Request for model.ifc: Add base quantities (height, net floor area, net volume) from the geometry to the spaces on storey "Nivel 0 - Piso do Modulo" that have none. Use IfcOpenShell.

First a look at what the model holds.

```python
import ifcopenshell
import ifcopenshell.util.element
import ifcopenshell.util.unit

model = ifcopenshell.open("model.ifc")
print(model.schema)
for unit_type in ("LENGTHUNIT", "AREAUNIT", "VOLUMEUNIT"):
    print(unit_type, ifcopenshell.util.unit.calculate_unit_scale(model, unit_type))
storey = next(s for s in model.by_type("IfcBuildingStorey") if s.Name == "Nivel 0 - Piso do Modulo")
spaces = [e for e in ifcopenshell.util.element.get_decomposition(storey) if e.is_a("IfcSpace")]
for e in sorted(spaces, key=lambda e: e.id()):
    print(e.id(), e.is_a(), e.Name, list(ifcopenshell.util.element.get_psets(e, qtos_only=True)), sep=" | ")
```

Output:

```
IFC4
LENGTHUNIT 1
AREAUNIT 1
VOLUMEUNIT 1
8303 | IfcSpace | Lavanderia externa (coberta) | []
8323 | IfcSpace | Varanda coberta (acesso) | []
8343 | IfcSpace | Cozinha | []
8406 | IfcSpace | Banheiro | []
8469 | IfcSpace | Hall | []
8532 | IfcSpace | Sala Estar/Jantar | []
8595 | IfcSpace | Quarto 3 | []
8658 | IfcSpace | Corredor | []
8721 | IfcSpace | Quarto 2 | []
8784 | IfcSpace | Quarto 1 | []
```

```python
import ifcopenshell
import ifcopenshell.api.pset
import ifcopenshell.geom
import ifcopenshell.util.element
import ifcopenshell.util.shape
import ifcopenshell.util.unit

model = ifcopenshell.open("model.ifc")
unit_scale = ifcopenshell.util.unit.calculate_unit_scale(model)
area_scale = ifcopenshell.util.unit.calculate_unit_scale(model, "AREAUNIT")
volume_scale = ifcopenshell.util.unit.calculate_unit_scale(model, "VOLUMEUNIT")
settings = ifcopenshell.geom.settings()

storey = next(s for s in model.by_type("IfcBuildingStorey") if s.Name == "Nivel 0 - Piso do Modulo")
spaces = [e for e in ifcopenshell.util.element.get_decomposition(storey) if e.is_a("IfcSpace")]

for e in sorted(spaces, key=lambda e: e.id()):
    if ifcopenshell.util.element.get_psets(e, qtos_only=True, should_inherit=False):
        continue
    # Geometry comes back in metres, in the element's own axes.
    shape = ifcopenshell.geom.create_shape(settings, e)
    values = {
        "Height": ifcopenshell.util.shape.get_z(shape.geometry) / unit_scale,
        "NetFloorArea": ifcopenshell.util.shape.get_footprint_area(shape.geometry) / area_scale,
        "NetVolume": ifcopenshell.util.shape.get_volume(shape.geometry) / volume_scale,
    }
    qto = ifcopenshell.api.pset.add_qto(model, product=e, name="Qto_SpaceBaseQuantities")
    ifcopenshell.api.pset.edit_qto(model, qto=qto, properties=values)
    print(e.id(), {k: round(v, 3) for k, v in values.items()})

model.write("model-out.ifc")
```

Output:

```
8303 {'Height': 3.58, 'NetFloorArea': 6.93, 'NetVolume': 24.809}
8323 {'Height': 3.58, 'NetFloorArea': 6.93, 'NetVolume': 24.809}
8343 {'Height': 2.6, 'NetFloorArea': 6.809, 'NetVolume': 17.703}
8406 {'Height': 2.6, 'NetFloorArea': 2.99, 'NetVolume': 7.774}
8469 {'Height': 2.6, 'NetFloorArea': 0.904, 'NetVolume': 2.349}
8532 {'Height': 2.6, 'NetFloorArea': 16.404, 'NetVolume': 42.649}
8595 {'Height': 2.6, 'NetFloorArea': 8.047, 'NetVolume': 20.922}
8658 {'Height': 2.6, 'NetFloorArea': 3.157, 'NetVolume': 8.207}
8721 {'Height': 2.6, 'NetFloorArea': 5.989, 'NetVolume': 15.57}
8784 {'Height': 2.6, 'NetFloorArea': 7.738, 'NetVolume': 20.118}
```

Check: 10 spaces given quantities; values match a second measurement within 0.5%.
